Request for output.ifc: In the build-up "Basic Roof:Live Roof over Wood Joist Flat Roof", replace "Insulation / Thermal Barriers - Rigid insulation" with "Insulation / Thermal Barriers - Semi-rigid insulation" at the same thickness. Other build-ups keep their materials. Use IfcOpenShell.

First a look at what the model holds.

```python
import ifcopenshell
import ifcopenshell.util.element

model = ifcopenshell.open("output.ifc")
print(model.schema)
for layer_set in model.by_type("IfcMaterialLayerSet"):
    if layer_set.LayerSetName == "Basic Roof:Live Roof over Wood Joist Flat Roof":
        for layer in layer_set.MaterialLayers:
            print(layer.id(), layer.Material and layer.Material.Name, layer.LayerThickness, sep=" | ")
        print(len(ifcopenshell.util.element.get_elements_by_material(model, layer_set)), "elements and types use it")
print(sorted(m.Name for m in model.by_type("IfcMaterial") if m.Name)[:60])
```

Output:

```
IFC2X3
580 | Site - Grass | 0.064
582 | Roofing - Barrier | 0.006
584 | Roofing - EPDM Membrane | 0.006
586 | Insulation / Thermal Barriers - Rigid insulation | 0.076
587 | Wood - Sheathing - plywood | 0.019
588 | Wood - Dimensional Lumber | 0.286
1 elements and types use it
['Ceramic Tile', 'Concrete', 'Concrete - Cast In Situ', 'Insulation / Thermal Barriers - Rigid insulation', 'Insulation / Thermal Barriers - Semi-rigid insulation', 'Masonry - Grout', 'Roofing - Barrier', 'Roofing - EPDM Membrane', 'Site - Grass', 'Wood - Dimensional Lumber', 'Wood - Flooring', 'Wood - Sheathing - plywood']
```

```python
import ifcopenshell
import ifcopenshell.api.material

model = ifcopenshell.open("output.ifc")

layer_set = next(s for s in model.by_type("IfcMaterialLayerSet") if s.LayerSetName == "Basic Roof:Live Roof over Wood Joist Flat Roof")
layer = next(l for l in layer_set.MaterialLayers if l.Material and l.Material.Name == "Insulation / Thermal Barriers - Rigid insulation")
material = next(m for m in model.by_type("IfcMaterial") if m.Name == "Insulation / Thermal Barriers - Semi-rigid insulation")

# Point this one layer at the other material; renaming the old one would change it everywhere.
ifcopenshell.api.material.edit_layer(model, layer=layer, attributes={}, material=material)

print([l.Material.Name if l.Material else None for l in layer_set.MaterialLayers])

model.write("output-out.ifc")
```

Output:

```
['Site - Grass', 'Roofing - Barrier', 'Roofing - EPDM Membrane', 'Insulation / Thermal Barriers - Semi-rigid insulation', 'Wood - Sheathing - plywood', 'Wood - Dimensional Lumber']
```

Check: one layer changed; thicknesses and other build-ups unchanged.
